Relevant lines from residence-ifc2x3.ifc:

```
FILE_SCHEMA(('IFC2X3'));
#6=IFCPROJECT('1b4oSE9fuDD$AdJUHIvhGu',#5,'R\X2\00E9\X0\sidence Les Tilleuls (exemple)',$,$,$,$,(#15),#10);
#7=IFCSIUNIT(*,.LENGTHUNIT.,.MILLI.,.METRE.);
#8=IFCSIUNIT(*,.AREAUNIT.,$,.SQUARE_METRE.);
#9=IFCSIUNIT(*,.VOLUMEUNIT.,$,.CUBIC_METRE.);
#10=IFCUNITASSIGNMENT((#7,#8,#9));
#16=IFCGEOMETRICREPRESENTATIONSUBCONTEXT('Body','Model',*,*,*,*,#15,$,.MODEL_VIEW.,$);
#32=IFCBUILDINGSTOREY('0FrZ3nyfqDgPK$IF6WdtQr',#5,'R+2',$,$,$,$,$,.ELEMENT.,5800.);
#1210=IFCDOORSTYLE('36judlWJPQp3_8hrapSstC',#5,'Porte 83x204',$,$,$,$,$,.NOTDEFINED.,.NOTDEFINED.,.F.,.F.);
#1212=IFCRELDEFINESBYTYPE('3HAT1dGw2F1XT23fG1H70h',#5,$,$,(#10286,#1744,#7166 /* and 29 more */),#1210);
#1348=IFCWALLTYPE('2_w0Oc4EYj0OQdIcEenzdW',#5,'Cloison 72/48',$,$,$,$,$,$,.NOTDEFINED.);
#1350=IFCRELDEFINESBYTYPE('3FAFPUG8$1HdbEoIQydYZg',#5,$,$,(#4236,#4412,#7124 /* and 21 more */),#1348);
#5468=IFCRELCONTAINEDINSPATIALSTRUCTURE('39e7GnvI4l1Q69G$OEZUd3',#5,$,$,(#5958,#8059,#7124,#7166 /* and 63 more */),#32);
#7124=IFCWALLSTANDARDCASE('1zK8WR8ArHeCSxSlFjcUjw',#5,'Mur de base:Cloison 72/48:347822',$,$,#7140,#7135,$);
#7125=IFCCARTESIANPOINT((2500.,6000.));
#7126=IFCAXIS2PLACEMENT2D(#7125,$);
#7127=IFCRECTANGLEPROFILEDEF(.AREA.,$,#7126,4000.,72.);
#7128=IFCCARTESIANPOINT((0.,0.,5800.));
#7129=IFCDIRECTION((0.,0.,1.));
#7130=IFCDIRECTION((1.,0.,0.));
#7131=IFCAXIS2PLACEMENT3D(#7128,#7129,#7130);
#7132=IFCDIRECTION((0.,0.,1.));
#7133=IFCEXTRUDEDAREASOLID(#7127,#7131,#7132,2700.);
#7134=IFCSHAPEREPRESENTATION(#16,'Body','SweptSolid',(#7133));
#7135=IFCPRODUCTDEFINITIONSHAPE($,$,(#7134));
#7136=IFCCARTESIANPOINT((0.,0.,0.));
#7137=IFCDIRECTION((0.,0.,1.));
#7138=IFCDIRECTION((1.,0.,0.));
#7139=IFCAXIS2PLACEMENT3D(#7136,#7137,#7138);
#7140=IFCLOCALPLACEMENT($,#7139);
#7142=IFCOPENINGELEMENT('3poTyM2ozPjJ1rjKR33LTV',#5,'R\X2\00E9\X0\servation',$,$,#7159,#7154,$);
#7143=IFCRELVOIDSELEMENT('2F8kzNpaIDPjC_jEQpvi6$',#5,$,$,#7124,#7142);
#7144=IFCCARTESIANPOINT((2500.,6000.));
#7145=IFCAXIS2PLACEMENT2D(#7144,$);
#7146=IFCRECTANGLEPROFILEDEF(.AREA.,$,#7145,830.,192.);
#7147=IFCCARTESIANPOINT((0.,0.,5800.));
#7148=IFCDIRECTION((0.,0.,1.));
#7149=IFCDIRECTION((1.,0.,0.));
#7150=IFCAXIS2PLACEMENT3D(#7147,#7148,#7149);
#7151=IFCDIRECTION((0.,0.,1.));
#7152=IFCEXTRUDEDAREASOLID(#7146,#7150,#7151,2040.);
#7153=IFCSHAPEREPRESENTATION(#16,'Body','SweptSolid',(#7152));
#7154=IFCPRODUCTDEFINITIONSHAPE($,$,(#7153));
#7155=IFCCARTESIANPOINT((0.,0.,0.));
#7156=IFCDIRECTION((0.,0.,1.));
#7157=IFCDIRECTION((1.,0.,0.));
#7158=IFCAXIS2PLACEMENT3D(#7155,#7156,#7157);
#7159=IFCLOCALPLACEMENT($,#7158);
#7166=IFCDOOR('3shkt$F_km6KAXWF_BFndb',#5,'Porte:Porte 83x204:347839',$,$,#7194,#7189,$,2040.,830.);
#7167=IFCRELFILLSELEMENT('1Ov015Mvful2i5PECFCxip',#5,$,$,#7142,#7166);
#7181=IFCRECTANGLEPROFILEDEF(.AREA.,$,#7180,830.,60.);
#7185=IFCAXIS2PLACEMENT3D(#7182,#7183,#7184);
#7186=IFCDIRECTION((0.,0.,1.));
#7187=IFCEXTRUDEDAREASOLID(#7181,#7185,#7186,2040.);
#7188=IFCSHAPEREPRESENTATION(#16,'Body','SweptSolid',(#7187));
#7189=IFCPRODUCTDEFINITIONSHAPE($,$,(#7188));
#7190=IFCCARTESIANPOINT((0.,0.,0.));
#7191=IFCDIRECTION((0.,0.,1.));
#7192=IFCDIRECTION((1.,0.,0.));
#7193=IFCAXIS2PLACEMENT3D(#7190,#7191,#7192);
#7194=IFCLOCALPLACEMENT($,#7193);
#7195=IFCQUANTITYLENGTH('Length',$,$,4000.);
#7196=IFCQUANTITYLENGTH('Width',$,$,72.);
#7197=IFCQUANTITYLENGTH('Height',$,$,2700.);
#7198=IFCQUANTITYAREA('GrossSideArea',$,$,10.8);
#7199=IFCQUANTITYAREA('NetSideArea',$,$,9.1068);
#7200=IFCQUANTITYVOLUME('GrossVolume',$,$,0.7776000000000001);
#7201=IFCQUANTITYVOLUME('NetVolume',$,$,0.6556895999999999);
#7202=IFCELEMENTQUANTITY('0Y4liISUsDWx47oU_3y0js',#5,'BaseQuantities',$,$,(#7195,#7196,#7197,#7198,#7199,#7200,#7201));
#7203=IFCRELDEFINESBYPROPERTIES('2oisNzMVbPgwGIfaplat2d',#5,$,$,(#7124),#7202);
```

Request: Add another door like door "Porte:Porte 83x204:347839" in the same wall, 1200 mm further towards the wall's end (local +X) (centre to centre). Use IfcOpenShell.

```python
import ifcopenshell
import ifcopenshell.api.feature
import ifcopenshell.api.geometry
import ifcopenshell.api.pset
import ifcopenshell.api.root
import ifcopenshell.geom
import ifcopenshell.util.element
import ifcopenshell.util.placement
import ifcopenshell.util.shape
import ifcopenshell.util.unit

model = ifcopenshell.open("residence-ifc2x3.ifc")
area_scale = ifcopenshell.util.unit.calculate_unit_scale(model, "AREAUNIT")
volume_scale = ifcopenshell.util.unit.calculate_unit_scale(model, "VOLUMEUNIT")
settings = ifcopenshell.geom.settings()


def volume(element):
    """Net volume in cubic metres, openings subtracted."""
    shape = ifcopenshell.geom.create_shape(settings, element)
    return ifcopenshell.util.shape.get_volume(shape.geometry)


def reuse_history(source, copy):
    """copy_class also copies each property set's owner history, people and application; keep the originals."""
    for rel in copy.IsDefinedBy:
        if rel.is_a("IfcRelDefinesByProperties") and (history := rel.RelatingPropertyDefinition.OwnerHistory):
            rel.RelatingPropertyDefinition.OwnerHistory = source.OwnerHistory
            ifcopenshell.util.element.remove_deep2(model, history)


door = model.by_guid("3shkt$F_km6KAXWF_BFndb")
opening = door.FillsVoids[0].RelatingOpeningElement
wall = opening.VoidsElements[0].RelatingBuildingElement
before = volume(wall)
shift = ifcopenshell.util.placement.get_local_placement(wall.ObjectPlacement)[:3, 0] * 1200.0

# copy_class copies the void relationship, type, container and properties, but no geometry.
new_opening = ifcopenshell.api.root.copy_class(model, product=opening)
new_opening.Representation = ifcopenshell.util.element.copy_deep(
    model, opening.Representation, exclude=["IfcGeometricRepresentationContext", "IfcRepresentationMap"]
)
reuse_history(opening, new_opening)
new_door = ifcopenshell.api.root.copy_class(model, product=door)
new_door.Representation = ifcopenshell.util.element.copy_deep(
    model, door.Representation, exclude=["IfcGeometricRepresentationContext", "IfcRepresentationMap"]
)
new_door.Name = "Porte:Porte 83x204"
reuse_history(door, new_door)
fills = ifcopenshell.api.feature.add_filling(model, opening=new_opening, element=new_door)
fills.OwnerHistory = new_door.OwnerHistory  # required in IFC2X3

for old, new in ((opening, new_opening), (door, new_door)):
    matrix = ifcopenshell.util.placement.get_local_placement(old.ObjectPlacement)
    matrix[:3, 3] += shift
    ifcopenshell.api.geometry.edit_object_placement(model, product=new, matrix=matrix, is_si=False)

after = volume(wall)
thickness = 0.072  # wall thickness in metres

# Update the wall's stored quantities.
qto = model.by_id(ifcopenshell.util.element.get_pset(wall, "BaseQuantities", should_inherit=False)["id"])
ifcopenshell.api.pset.edit_qto(model, qto=qto, properties={
    "NetSideArea": after / thickness / area_scale,
    "NetVolume": after / volume_scale,
})

print(f"wall volume {before:.3f} -> {after:.3f} m3")

model.write("residence-ifc2x3_edited.ifc")
```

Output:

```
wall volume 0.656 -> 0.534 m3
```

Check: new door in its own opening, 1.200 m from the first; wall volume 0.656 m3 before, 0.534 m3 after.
